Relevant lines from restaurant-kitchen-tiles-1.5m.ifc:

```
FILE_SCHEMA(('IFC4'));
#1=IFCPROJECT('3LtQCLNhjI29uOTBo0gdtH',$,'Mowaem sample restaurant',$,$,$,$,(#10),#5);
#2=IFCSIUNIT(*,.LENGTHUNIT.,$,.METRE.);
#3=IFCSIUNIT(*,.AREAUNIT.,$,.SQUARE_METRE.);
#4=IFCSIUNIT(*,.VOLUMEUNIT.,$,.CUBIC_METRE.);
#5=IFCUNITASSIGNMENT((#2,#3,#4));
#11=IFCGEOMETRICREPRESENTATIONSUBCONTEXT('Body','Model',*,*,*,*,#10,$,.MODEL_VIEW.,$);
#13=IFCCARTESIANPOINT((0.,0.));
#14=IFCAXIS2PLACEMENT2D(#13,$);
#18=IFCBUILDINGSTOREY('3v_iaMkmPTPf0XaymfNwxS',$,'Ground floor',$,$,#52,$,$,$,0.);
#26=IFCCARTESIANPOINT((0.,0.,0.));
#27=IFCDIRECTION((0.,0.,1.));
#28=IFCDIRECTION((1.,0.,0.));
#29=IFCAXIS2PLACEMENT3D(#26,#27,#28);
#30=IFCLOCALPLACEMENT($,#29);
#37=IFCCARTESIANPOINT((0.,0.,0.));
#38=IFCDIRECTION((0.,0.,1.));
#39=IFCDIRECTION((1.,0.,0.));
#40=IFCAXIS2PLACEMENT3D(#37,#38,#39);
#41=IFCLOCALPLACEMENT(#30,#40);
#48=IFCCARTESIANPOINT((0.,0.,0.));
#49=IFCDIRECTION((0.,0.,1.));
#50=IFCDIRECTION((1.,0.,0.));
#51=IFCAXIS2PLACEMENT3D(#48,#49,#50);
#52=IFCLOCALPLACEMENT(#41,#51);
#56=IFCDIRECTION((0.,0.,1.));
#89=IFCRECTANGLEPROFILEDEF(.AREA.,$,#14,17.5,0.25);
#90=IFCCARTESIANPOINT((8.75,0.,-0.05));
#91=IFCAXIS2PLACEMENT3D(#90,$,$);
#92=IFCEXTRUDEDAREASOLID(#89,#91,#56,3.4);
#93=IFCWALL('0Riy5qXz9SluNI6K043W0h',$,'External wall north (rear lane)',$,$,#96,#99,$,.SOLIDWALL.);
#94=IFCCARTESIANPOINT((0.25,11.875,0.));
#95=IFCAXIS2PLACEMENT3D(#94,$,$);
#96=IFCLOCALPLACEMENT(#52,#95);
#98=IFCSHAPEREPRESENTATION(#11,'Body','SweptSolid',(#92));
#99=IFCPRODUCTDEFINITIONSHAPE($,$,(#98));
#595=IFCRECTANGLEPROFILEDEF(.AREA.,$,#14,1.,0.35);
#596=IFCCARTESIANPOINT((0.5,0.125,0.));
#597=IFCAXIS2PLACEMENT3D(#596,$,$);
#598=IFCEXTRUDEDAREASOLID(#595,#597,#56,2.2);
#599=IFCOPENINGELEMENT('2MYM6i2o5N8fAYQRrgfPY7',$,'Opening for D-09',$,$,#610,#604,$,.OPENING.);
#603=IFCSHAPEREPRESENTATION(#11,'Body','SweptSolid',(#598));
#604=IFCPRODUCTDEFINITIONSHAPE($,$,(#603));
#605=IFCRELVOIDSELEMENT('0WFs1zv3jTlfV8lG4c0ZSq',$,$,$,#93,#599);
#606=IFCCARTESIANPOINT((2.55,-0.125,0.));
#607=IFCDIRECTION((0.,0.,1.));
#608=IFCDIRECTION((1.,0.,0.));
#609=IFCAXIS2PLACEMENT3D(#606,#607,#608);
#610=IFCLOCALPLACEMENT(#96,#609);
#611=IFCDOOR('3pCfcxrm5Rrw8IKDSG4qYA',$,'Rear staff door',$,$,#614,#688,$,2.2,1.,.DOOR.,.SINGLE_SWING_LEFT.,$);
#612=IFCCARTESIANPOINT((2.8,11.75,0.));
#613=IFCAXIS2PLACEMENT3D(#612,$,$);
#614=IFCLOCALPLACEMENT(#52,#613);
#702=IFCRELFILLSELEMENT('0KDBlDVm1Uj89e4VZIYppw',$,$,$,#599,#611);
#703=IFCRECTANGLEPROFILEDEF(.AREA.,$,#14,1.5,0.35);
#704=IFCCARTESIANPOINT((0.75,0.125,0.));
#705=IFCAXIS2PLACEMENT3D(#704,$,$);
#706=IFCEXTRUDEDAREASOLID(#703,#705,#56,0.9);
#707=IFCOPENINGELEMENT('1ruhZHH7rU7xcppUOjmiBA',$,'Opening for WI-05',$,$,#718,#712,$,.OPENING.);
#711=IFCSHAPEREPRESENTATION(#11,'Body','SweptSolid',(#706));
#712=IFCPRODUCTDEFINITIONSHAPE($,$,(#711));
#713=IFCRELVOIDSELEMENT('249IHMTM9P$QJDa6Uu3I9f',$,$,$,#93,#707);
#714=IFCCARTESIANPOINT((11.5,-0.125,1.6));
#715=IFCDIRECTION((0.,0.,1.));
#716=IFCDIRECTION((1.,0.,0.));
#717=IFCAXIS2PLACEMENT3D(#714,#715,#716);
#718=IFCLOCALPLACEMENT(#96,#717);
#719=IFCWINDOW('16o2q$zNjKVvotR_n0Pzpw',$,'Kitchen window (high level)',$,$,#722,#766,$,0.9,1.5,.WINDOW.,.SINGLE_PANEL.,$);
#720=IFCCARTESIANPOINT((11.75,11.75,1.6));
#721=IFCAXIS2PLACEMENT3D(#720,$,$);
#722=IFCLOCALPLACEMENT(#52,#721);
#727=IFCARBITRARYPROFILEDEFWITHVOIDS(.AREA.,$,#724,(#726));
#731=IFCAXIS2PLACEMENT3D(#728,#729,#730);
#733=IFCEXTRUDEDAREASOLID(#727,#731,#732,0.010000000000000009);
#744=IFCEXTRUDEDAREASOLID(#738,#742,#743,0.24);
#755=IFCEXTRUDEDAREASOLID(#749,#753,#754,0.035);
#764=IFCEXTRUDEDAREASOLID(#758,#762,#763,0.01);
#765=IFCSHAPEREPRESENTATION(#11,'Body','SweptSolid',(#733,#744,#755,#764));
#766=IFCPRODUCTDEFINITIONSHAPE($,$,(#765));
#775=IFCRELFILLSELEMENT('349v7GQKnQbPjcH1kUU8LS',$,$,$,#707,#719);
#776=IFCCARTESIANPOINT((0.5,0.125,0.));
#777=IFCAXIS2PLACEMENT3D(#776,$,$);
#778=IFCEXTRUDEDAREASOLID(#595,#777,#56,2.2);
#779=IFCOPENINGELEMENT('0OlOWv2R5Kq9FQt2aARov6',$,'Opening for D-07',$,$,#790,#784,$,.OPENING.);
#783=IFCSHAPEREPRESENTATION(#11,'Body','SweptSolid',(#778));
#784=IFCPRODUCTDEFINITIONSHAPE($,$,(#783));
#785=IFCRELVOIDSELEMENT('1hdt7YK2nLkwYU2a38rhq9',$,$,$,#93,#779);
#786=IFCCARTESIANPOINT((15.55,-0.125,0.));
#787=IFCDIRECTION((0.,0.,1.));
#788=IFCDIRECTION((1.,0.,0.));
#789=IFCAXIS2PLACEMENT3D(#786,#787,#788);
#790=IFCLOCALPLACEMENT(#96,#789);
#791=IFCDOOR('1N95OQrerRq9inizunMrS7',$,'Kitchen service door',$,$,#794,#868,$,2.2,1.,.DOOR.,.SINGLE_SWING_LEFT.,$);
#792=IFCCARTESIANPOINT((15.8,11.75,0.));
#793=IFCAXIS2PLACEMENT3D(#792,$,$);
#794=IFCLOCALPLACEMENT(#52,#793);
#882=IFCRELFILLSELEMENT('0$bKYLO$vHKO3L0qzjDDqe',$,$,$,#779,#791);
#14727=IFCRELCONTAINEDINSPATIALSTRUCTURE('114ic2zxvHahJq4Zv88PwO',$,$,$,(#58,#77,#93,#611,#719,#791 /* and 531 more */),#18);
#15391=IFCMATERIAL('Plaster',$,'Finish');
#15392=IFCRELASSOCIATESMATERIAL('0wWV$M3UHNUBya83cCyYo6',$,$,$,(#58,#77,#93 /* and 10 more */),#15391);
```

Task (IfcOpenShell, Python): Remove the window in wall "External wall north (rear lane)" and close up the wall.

```python
import ifcopenshell
import ifcopenshell.api.feature
import ifcopenshell.api.root
import ifcopenshell.geom
import ifcopenshell.util.shape

model = ifcopenshell.open("restaurant-kitchen-tiles-1.5m.ifc")
settings = ifcopenshell.geom.settings()


def volume(element):
    """Net volume in cubic metres, openings subtracted."""
    shape = ifcopenshell.geom.create_shape(settings, element)
    return ifcopenshell.util.shape.get_volume(shape.geometry)


window = model.by_guid("16o2q$zNjKVvotR_n0Pzpw")
opening = window.FillsVoids[0].RelatingOpeningElement
wall = opening.VoidsElements[0].RelatingBuildingElement
before = volume(wall)

ifcopenshell.api.root.remove_product(model, product=window)
ifcopenshell.api.feature.remove_feature(model, feature=opening)

after = volume(wall)

print(f"wall volume {before:.3f} -> {after:.3f} m3")

model.write("restaurant-kitchen-tiles-1.5m_updated.ifc")
```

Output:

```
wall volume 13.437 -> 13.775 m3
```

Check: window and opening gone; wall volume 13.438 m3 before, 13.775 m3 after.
